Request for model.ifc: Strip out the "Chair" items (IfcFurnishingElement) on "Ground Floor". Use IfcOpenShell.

First a look at what the model holds.

```python
import ifcopenshell
import ifcopenshell.util.element

model = ifcopenshell.open("model.ifc")
print(model.schema)
storey = next(s for s in model.by_type("IfcBuildingStorey") if s.Name == "Ground Floor")
furniture = [e for e in ifcopenshell.util.element.get_decomposition(storey) if e.is_a("IfcFurnishingElement")]
seen = {}
for e in furniture:
    element_type = ifcopenshell.util.element.get_type(e)
    name = element_type.Name if element_type not in (None, e) else None
    seen[name] = seen.get(name, 0) + 1
for name, count in sorted(seen.items(), key=str):
    print(count, "x", name)
```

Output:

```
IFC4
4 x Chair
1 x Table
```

```python
import ifcopenshell
import ifcopenshell.api.root
import ifcopenshell.util.element

model = ifcopenshell.open("model.ifc")

storey = next(s for s in model.by_type("IfcBuildingStorey") if s.Name == "Ground Floor")
furniture = [e for e in ifcopenshell.util.element.get_decomposition(storey) if e.is_a("IfcFurnishingElement")]
targets = [e for e in furniture if (t := ifcopenshell.util.element.get_type(e)) not in (None, e) and t.Name == "Chair"]

for e in targets:
    ifcopenshell.api.root.remove_product(model, product=e)
print(len(targets), "removed")

model.write("model_rev.ifc")
```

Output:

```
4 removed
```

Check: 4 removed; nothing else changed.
